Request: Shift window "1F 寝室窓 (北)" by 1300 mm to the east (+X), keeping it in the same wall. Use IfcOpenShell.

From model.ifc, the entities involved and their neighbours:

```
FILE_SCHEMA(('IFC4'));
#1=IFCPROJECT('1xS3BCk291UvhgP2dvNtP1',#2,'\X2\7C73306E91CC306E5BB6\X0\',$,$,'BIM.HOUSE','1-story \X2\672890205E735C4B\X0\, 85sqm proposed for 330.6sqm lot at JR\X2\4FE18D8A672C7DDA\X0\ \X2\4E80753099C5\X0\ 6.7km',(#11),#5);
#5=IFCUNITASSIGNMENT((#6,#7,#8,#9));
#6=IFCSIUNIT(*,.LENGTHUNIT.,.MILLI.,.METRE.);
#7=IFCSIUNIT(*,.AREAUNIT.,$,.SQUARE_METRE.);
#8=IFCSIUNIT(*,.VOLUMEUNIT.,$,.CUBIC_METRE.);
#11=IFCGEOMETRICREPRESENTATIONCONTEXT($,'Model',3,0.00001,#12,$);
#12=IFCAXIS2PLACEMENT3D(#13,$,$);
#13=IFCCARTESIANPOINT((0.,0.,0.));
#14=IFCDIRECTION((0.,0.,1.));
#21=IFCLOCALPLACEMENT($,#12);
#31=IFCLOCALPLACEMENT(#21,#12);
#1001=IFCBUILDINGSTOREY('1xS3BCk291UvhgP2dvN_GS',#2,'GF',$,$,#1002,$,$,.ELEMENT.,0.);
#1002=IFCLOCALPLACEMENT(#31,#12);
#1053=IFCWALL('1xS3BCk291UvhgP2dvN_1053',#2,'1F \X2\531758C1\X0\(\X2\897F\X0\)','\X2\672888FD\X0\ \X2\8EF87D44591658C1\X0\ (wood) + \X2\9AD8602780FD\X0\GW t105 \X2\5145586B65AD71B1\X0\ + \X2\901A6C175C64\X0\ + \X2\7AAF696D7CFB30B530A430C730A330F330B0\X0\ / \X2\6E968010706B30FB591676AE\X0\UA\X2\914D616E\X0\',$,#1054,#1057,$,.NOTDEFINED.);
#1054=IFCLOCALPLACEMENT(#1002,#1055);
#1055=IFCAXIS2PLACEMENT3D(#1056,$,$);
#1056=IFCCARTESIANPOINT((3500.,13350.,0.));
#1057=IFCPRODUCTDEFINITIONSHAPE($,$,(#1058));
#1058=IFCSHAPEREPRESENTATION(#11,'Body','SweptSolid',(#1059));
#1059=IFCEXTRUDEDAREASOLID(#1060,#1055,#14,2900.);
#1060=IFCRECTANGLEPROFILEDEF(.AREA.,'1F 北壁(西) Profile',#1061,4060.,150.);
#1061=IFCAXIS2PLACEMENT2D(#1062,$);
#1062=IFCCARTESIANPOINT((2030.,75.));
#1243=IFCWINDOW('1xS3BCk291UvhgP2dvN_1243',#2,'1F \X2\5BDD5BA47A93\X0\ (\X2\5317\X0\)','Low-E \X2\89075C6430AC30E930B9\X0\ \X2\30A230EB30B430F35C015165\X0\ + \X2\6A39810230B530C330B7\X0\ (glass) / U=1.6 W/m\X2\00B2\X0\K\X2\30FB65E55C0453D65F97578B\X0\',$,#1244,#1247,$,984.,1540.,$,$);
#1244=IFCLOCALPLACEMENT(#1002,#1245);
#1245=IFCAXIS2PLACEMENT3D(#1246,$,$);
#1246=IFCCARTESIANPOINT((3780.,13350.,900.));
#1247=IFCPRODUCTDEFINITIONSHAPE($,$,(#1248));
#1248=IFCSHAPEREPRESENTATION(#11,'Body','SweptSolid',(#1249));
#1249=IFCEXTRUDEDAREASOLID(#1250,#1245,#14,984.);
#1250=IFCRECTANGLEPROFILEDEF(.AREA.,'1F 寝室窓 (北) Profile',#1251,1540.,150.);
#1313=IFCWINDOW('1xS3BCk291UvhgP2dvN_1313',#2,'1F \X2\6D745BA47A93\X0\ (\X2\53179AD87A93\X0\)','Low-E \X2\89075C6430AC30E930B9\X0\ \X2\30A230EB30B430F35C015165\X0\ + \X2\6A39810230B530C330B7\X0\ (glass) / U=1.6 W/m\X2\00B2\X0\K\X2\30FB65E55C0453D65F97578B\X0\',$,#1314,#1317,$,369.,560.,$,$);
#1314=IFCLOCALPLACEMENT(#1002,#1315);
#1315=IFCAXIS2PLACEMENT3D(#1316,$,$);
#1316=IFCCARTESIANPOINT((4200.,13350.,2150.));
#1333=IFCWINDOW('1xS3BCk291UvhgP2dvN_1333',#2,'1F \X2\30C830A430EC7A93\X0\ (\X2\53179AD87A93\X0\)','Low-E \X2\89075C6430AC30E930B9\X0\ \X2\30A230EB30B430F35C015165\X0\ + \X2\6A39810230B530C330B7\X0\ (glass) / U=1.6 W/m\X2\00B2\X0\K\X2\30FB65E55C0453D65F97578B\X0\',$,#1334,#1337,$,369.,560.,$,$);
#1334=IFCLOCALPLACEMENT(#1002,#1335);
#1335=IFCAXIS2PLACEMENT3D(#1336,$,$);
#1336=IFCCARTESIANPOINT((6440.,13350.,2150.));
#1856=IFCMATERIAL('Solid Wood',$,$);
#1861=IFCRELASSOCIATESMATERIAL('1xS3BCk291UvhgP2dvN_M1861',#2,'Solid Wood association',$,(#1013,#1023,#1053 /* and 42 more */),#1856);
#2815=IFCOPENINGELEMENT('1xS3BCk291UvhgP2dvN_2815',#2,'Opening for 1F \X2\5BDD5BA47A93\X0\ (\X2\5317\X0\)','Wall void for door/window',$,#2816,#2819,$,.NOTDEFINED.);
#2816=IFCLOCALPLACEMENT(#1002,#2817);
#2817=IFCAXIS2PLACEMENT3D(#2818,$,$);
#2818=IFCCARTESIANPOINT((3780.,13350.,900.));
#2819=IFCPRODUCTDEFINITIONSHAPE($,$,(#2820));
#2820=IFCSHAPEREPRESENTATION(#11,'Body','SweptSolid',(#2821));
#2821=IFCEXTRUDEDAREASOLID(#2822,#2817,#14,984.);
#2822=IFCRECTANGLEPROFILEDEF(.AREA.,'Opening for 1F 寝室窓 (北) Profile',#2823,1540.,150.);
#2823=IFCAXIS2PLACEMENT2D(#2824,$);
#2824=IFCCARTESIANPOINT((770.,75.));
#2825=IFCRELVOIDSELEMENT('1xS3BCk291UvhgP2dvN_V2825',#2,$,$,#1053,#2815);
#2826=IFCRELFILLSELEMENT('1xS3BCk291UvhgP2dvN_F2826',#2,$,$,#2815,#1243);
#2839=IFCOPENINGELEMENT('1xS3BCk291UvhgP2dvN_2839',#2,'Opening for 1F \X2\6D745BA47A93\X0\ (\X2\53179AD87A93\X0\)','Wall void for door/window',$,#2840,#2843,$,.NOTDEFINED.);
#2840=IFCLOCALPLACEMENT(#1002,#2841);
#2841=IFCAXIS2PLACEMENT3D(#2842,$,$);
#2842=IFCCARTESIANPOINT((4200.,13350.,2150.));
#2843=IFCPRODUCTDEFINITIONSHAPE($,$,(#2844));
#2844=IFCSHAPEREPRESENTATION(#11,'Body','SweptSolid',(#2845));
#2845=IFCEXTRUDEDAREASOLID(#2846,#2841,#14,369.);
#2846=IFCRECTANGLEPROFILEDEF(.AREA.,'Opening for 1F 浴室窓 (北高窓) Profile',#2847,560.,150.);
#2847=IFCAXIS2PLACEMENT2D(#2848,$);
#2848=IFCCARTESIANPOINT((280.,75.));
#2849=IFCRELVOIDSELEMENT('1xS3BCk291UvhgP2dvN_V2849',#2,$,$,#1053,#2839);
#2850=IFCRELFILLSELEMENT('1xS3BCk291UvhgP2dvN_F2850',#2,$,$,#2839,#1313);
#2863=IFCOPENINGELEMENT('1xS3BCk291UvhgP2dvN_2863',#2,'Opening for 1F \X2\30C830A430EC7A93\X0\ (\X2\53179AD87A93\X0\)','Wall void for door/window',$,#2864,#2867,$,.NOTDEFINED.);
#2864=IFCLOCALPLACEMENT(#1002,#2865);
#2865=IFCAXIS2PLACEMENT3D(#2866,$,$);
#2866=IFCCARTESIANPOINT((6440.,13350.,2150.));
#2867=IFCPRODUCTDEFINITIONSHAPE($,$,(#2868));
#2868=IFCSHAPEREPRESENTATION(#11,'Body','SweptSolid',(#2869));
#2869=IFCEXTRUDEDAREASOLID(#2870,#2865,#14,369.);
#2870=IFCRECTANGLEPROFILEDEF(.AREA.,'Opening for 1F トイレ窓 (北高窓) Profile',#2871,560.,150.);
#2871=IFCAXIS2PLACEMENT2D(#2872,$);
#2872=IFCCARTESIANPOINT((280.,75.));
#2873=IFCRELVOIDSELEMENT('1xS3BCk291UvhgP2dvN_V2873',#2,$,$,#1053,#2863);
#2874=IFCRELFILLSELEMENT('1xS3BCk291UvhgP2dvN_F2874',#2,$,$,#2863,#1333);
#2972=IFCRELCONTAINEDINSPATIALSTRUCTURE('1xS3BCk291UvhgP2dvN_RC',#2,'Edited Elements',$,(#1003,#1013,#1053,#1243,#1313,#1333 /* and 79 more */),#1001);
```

```python
import ifcopenshell
import ifcopenshell.api.geometry
import ifcopenshell.util.placement
import ifcopenshell.util.unit

model = ifcopenshell.open("model.ifc")
unit_scale = ifcopenshell.util.unit.calculate_unit_scale(model)

window = model.by_guid("1xS3BCk291UvhgP2dvN_1243")
opening = window.FillsVoids[0].RelatingOpeningElement
wall = opening.VoidsElements[0].RelatingBuildingElement

wall_matrix = ifcopenshell.util.placement.get_local_placement(wall.ObjectPlacement)
shift = wall_matrix[:3, 0] * 1.3 / unit_scale
before = ifcopenshell.util.placement.get_local_placement(window.ObjectPlacement)[:3, 3].copy()

# The window is not placed relative to its opening, so move both.
for product in (opening, window):
    matrix = ifcopenshell.util.placement.get_local_placement(product.ObjectPlacement)
    matrix[:3, 3] += shift
    ifcopenshell.api.geometry.edit_object_placement(model, product=product, matrix=matrix, is_si=False)

after = ifcopenshell.util.placement.get_local_placement(window.ObjectPlacement)[:3, 3]
print("window moved by", (after - before).round(3) + 0.0)

model.write("model_edited.ifc")
```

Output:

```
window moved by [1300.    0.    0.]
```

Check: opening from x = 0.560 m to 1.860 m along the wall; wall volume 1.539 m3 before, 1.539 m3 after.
